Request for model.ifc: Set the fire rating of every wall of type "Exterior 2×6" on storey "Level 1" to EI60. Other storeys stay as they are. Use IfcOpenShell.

First a look at what the model holds.

```python
import ifcopenshell
import ifcopenshell.util.element

model = ifcopenshell.open("model.ifc")
print(model.schema)
storey = next(s for s in model.by_type("IfcBuildingStorey") if s.Name == "Level 1")
walls = [e for e in ifcopenshell.util.element.get_decomposition(storey) if e.is_a("IfcWall")]
seen = {}
for e in walls:
    element_type = ifcopenshell.util.element.get_type(e)
    key = (element_type.Name if element_type != e and element_type else None, ifcopenshell.util.element.get_pset(e, "Pset_WallCommon", "FireRating"))
    seen[key] = seen.get(key, 0) + 1
for (name, value), count in sorted(seen.items(), key=str):
    print(count, "x", name, "|", value)
```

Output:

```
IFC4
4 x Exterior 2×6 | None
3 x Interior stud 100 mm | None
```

```python
import ifcopenshell
import ifcopenshell.api.pset
import ifcopenshell.util.element

model = ifcopenshell.open("model.ifc")

storey = next(s for s in model.by_type("IfcBuildingStorey") if s.Name == "Level 1")
walls = [e for e in ifcopenshell.util.element.get_decomposition(storey) if e.is_a("IfcWall")]

count = 0
for e in walls:
    element_type = ifcopenshell.util.element.get_type(e)
    if element_type in (None, e) or element_type.Name != "Exterior 2×6":
        continue
    # add_pset returns the element's existing set when there is one.
    pset = ifcopenshell.api.pset.add_pset(model, product=e, name="Pset_WallCommon")
    ifcopenshell.api.pset.edit_pset(model, pset=pset, properties={"FireRating": "EI60"})
    count += 1

print(count, "walls updated")

model.write("model_rev.ifc")
```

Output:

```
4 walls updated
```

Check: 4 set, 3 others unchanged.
